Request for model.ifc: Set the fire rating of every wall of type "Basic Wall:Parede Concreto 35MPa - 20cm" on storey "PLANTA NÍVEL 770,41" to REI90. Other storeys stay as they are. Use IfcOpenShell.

First a look at what the model holds.

```python
import ifcopenshell
import ifcopenshell.util.element

model = ifcopenshell.open("model.ifc")
print(model.schema)
storey = next(s for s in model.by_type("IfcBuildingStorey") if s.Name == "PLANTA NÍVEL 770,41")
walls = [e for e in ifcopenshell.util.element.get_decomposition(storey) if e.is_a("IfcWall")]
seen = {}
for e in walls:
    element_type = ifcopenshell.util.element.get_type(e)
    key = (element_type.Name if element_type != e and element_type else None, ifcopenshell.util.element.get_pset(e, "Pset_WallCommon", "FireRating"))
    seen[key] = seen.get(key, 0) + 1
for (name, value), count in sorted(seen.items(), key=str):
    print(count, "x", name, "|", value)
```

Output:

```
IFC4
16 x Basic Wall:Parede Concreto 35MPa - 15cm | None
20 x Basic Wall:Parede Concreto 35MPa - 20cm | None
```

```python
import ifcopenshell
import ifcopenshell.api.pset
import ifcopenshell.util.element

model = ifcopenshell.open("model.ifc")

storey = next(s for s in model.by_type("IfcBuildingStorey") if s.Name == "PLANTA NÍVEL 770,41")
walls = [e for e in ifcopenshell.util.element.get_decomposition(storey) if e.is_a("IfcWall")]

count = 0
for e in walls:
    element_type = ifcopenshell.util.element.get_type(e)
    if element_type in (None, e) or element_type.Name != "Basic Wall:Parede Concreto 35MPa - 20cm":
        continue
    # add_pset returns the element's existing set when there is one.
    pset = ifcopenshell.api.pset.add_pset(model, product=e, name="Pset_WallCommon")
    ifcopenshell.api.pset.edit_pset(model, pset=pset, properties={"FireRating": "REI90"})
    count += 1

print(count, "walls updated")

model.write("model_rev.ifc")
```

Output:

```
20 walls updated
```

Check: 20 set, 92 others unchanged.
